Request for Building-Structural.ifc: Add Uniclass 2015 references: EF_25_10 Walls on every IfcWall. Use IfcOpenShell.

First a look at what the model holds.

```python
import ifcopenshell

model = ifcopenshell.open("Building-Structural.ifc")
print(model.schema)
print("classifications:", [c.Name for c in model.by_type("IfcClassification")])
for ifc_class in ("IfcDoor", "IfcRoof", "IfcStair", "IfcWall", "IfcWindow"):
    print(ifc_class, len(model.by_type(ifc_class)))
```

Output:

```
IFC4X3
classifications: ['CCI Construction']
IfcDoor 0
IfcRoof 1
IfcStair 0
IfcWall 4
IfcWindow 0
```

```python
import ifcopenshell
import ifcopenshell.api.classification

model = ifcopenshell.open("Building-Structural.ifc")

system = ifcopenshell.api.classification.add_classification(model, classification="Uniclass 2015")

codes = {
    "IfcWall": ("EF_25_10", "Walls"),
}
for ifc_class, (code, name) in codes.items():
    products = model.by_type(ifc_class)
    ifcopenshell.api.classification.add_reference(
        model, products=products, classification=system, identification=code, name=name
    )
    print(code, len(products))

model.write("Building-Structural_rev.ifc")
```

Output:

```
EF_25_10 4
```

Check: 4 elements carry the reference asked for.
